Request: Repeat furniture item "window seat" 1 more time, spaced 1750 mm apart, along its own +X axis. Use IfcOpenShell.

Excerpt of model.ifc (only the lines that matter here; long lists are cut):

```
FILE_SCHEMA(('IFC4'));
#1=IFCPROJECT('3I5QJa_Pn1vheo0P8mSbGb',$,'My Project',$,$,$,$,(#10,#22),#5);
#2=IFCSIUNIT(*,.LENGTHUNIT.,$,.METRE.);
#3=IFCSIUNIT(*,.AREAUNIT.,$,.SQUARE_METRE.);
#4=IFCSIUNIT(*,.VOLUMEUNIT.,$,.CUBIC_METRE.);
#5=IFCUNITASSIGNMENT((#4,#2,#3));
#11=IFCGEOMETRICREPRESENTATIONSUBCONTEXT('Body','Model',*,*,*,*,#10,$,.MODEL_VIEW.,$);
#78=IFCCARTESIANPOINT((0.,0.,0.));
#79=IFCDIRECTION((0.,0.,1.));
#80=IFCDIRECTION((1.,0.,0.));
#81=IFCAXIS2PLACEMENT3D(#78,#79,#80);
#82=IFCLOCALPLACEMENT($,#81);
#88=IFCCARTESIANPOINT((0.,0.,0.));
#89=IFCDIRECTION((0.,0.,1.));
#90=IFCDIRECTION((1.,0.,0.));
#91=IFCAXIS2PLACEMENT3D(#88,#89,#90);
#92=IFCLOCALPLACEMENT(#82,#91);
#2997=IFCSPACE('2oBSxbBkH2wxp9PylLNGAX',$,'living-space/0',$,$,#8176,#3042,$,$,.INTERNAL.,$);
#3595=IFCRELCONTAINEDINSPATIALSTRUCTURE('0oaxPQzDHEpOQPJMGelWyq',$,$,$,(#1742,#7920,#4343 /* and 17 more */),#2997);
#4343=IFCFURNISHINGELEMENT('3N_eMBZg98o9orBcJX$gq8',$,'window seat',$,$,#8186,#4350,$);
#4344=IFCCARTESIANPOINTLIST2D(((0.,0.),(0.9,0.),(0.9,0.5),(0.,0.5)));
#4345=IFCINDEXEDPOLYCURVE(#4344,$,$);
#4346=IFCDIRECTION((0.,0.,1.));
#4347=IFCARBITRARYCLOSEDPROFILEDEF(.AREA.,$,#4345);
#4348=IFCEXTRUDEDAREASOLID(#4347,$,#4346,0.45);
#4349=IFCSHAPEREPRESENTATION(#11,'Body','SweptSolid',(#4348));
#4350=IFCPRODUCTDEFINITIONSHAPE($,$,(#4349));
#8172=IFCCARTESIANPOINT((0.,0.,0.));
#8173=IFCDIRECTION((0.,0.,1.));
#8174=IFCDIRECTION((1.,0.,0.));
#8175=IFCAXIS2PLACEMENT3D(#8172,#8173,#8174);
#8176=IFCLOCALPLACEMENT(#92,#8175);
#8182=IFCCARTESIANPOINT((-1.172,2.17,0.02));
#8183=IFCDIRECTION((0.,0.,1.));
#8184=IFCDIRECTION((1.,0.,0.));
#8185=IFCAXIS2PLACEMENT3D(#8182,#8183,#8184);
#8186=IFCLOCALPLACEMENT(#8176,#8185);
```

```python
import ifcopenshell
import ifcopenshell.api.geometry
import ifcopenshell.api.root
import ifcopenshell.util.element
import ifcopenshell.util.placement
import ifcopenshell.util.unit

model = ifcopenshell.open("model.ifc")
unit_scale = ifcopenshell.util.unit.calculate_unit_scale(model)

source = model.by_id(4343)
base = ifcopenshell.util.placement.get_local_placement(source.ObjectPlacement)
step = base[:3, 0] * 1.75 / unit_scale

for i in range(1, 2):
    copy = ifcopenshell.api.root.copy_class(model, product=source)
    copy.Representation = ifcopenshell.util.element.copy_deep(
        model, source.Representation, exclude=["IfcGeometricRepresentationContext", "IfcRepresentationMap"]
    )
    matrix = base.copy()
    matrix[:3, 3] += i * step
    print("added at", matrix[:3, 3].round(3) + 0.0)
    ifcopenshell.api.geometry.edit_object_placement(model, product=copy, matrix=matrix, is_si=False)

model.write("model-out.ifc")
```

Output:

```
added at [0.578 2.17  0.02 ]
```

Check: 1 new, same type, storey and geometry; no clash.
